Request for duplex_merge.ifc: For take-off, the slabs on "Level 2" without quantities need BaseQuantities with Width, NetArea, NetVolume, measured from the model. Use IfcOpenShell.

First a look at what the model holds.

```python
import ifcopenshell
import ifcopenshell.util.element
import ifcopenshell.util.unit

model = ifcopenshell.open("duplex_merge.ifc")
print(model.schema)
for unit_type in ("LENGTHUNIT", "AREAUNIT", "VOLUMEUNIT"):
    print(unit_type, ifcopenshell.util.unit.calculate_unit_scale(model, unit_type))
storey = next(s for s in model.by_type("IfcBuildingStorey") if s.Name == "Level 2")
slabs = [e for e in ifcopenshell.util.element.get_decomposition(storey) if e.is_a("IfcSlab")]
for e in sorted(slabs, key=lambda e: e.id()):
    print(e.id(), e.is_a(), e.Name, list(ifcopenshell.util.element.get_psets(e, qtos_only=True)), sep=" | ")
```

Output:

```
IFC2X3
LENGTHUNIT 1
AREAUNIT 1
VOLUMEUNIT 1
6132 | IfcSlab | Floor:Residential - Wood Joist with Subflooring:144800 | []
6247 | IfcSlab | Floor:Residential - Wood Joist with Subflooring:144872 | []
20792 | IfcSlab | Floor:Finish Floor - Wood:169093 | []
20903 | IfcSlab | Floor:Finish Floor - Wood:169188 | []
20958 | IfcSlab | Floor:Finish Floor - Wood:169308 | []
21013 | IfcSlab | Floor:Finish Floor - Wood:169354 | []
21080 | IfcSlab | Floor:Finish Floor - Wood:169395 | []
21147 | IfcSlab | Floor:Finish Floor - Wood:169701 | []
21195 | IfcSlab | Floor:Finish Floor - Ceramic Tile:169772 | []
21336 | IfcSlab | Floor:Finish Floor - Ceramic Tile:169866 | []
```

```python
import ifcopenshell
import ifcopenshell.api.pset
import ifcopenshell.geom
import ifcopenshell.util.element
import ifcopenshell.util.shape
import ifcopenshell.util.unit

model = ifcopenshell.open("duplex_merge.ifc")
unit_scale = ifcopenshell.util.unit.calculate_unit_scale(model)
area_scale = ifcopenshell.util.unit.calculate_unit_scale(model, "AREAUNIT")
volume_scale = ifcopenshell.util.unit.calculate_unit_scale(model, "VOLUMEUNIT")
settings = ifcopenshell.geom.settings()

storey = next(s for s in model.by_type("IfcBuildingStorey") if s.Name == "Level 2")
slabs = [e for e in ifcopenshell.util.element.get_decomposition(storey) if e.is_a("IfcSlab")]

for e in sorted(slabs, key=lambda e: e.id()):
    if ifcopenshell.util.element.get_psets(e, qtos_only=True, should_inherit=False):
        continue
    # Geometry comes back in metres, in the element's own axes.
    shape = ifcopenshell.geom.create_shape(settings, e)
    values = {
        "Width": ifcopenshell.util.shape.get_z(shape.geometry) / unit_scale,
        "NetArea": ifcopenshell.util.shape.get_footprint_area(shape.geometry) / area_scale,
        "NetVolume": ifcopenshell.util.shape.get_volume(shape.geometry) / volume_scale,
    }
    qto = ifcopenshell.api.pset.add_qto(model, product=e, name="BaseQuantities")
    ifcopenshell.api.pset.edit_qto(model, qto=qto, properties=values)
    print(e.id(), {k: round(v, 3) for k, v in values.items()})

model.write("duplex_merge_edited.ifc")
```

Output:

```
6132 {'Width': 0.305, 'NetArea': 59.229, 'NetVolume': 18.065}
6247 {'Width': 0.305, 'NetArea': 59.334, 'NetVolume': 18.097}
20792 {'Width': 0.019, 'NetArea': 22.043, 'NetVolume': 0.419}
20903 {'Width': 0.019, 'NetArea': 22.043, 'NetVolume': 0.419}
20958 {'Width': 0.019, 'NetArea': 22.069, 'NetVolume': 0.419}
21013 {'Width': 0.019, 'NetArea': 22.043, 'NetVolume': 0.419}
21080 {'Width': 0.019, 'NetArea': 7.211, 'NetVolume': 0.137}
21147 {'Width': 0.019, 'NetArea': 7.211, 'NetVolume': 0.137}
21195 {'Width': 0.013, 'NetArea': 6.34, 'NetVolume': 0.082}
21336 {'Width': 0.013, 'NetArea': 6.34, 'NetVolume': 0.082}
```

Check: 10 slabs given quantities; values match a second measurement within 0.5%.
